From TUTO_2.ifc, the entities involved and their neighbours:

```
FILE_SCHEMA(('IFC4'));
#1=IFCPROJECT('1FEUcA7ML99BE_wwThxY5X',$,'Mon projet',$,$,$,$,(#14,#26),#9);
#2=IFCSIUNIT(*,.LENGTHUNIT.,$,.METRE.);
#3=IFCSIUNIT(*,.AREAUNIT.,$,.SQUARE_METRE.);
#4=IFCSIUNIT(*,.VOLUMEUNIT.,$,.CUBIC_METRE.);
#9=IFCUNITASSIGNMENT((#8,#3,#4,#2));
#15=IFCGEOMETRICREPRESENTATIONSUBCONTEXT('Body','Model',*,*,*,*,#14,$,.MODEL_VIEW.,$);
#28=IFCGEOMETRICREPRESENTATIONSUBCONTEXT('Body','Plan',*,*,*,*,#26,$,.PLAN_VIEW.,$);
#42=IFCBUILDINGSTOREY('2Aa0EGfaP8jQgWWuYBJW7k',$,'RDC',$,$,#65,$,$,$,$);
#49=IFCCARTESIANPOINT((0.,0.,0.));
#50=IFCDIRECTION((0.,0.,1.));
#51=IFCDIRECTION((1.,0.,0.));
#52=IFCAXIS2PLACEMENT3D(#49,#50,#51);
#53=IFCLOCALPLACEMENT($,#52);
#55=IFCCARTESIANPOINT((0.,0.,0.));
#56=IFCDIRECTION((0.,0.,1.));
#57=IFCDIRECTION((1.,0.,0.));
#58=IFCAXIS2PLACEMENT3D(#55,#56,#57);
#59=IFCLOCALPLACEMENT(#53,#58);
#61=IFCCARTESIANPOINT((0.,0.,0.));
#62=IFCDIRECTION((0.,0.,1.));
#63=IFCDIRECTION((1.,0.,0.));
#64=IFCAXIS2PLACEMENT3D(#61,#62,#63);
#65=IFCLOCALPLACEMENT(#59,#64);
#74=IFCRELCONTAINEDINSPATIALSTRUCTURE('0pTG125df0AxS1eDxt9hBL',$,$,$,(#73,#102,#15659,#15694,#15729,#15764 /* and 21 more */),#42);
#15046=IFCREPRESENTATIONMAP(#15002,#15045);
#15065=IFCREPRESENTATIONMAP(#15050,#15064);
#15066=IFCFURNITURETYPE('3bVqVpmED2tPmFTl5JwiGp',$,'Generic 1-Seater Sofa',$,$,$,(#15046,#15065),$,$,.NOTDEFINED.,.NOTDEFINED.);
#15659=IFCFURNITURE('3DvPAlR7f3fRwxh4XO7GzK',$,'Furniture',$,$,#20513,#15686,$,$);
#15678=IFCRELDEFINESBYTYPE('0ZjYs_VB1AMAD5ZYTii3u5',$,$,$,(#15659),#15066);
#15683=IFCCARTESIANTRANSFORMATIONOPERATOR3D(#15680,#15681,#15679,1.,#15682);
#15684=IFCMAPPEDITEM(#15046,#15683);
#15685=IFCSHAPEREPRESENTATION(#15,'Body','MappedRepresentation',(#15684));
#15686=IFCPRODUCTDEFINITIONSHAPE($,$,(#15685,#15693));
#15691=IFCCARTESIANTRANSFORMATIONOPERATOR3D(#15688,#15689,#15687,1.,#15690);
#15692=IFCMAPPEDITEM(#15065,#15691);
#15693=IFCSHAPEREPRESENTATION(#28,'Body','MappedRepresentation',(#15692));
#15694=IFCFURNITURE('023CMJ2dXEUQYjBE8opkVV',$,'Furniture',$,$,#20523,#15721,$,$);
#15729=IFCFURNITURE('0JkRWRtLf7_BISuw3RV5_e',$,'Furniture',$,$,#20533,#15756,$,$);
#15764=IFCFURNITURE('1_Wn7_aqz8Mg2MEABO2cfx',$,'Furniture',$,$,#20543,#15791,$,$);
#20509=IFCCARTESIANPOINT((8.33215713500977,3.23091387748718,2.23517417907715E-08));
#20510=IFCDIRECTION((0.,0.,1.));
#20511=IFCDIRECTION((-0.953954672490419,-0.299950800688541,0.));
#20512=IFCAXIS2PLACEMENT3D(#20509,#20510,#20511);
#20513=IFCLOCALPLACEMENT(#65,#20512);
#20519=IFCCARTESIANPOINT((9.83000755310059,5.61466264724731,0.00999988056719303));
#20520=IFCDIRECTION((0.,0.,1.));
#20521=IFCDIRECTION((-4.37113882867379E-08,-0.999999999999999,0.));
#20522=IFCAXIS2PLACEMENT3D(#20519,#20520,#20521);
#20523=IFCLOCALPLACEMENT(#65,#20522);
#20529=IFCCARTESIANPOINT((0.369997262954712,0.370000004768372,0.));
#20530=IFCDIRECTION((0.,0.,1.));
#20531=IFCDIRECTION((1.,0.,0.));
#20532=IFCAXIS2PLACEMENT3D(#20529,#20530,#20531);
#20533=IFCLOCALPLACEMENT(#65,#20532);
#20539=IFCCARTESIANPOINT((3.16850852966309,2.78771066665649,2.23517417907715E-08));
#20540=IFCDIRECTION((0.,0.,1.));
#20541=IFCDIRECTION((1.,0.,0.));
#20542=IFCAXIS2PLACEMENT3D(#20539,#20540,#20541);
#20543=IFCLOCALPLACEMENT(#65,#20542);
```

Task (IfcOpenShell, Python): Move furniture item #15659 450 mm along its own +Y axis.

```python
import ifcopenshell
import ifcopenshell.api.geometry
import ifcopenshell.util.placement

model = ifcopenshell.open("TUTO_2.ifc")

item = model.by_id(15659)
matrix = ifcopenshell.util.placement.get_local_placement(item.ObjectPlacement)
matrix[:3, 3] += matrix[:3, 1] * 0.45
ifcopenshell.api.geometry.edit_object_placement(model, product=item, matrix=matrix, is_si=False)

print(ifcopenshell.util.placement.get_local_placement(item.ObjectPlacement).round(3) + 0.0)

model.write("TUTO_2_updated.ifc")
```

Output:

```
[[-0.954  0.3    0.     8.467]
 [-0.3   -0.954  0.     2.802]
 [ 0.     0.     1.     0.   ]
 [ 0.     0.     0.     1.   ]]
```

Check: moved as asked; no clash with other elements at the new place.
